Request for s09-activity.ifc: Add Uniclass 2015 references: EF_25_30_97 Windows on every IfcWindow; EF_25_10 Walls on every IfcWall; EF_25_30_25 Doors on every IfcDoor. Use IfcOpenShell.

First a look at what the model holds.

```python
import ifcopenshell

model = ifcopenshell.open("s09-activity.ifc")
print(model.schema)
print("classifications:", [c.Name for c in model.by_type("IfcClassification")])
for ifc_class in ("IfcDoor", "IfcRoof", "IfcStair", "IfcWall", "IfcWindow"):
    print(ifc_class, len(model.by_type(ifc_class)))
```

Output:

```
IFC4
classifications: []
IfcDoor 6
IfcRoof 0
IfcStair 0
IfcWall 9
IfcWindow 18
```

```python
import ifcopenshell
import ifcopenshell.api.classification

model = ifcopenshell.open("s09-activity.ifc")

system = ifcopenshell.api.classification.add_classification(model, classification="Uniclass 2015")

codes = {
    "IfcWindow": ("EF_25_30_97", "Windows"),
    "IfcWall": ("EF_25_10", "Walls"),
    "IfcDoor": ("EF_25_30_25", "Doors"),
}
for ifc_class, (code, name) in codes.items():
    products = model.by_type(ifc_class)
    ifcopenshell.api.classification.add_reference(
        model, products=products, classification=system, identification=code, name=name
    )
    print(code, len(products))

model.write("s09-activity-out.ifc")
```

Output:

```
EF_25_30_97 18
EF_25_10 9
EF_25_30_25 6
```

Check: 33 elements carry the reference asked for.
